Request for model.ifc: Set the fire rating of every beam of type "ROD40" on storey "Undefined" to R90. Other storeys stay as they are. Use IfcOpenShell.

First a look at what the model holds.

```python
import ifcopenshell
import ifcopenshell.util.element

model = ifcopenshell.open("model.ifc")
print(model.schema)
storey = next(s for s in model.by_type("IfcBuildingStorey") if s.Name == "Undefined")
beams = [e for e in ifcopenshell.util.element.get_decomposition(storey) if e.is_a("IfcBeam")]
seen = {}
for e in beams:
    element_type = ifcopenshell.util.element.get_type(e)
    key = (element_type.Name if element_type != e and element_type else None, ifcopenshell.util.element.get_pset(e, "Pset_BeamCommon", "FireRating"))
    seen[key] = seen.get(key, 0) + 1
for (name, value), count in sorted(seen.items(), key=str):
    print(count, "x", name, "|", value)
```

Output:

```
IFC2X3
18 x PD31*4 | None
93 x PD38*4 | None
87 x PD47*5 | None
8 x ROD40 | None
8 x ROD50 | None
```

```python
import ifcopenshell
import ifcopenshell.api.pset
import ifcopenshell.util.element

model = ifcopenshell.open("model.ifc")

storey = next(s for s in model.by_type("IfcBuildingStorey") if s.Name == "Undefined")
beams = [e for e in ifcopenshell.util.element.get_decomposition(storey) if e.is_a("IfcBeam")]

count = 0
for e in beams:
    element_type = ifcopenshell.util.element.get_type(e)
    if element_type in (None, e) or element_type.Name != "ROD40":
        continue
    found = ifcopenshell.util.element.get_pset(e, "Pset_BeamCommon", should_inherit=False)
    if found:
        pset = model.by_id(found["id"])
        if len(ifcopenshell.util.element.get_elements_by_pset(pset)) > 1:
            pset = ifcopenshell.api.pset.unshare_pset(model, products=[e], pset=pset)[0]
    else:
        pset = ifcopenshell.api.pset.add_pset(model, product=e, name="Pset_BeamCommon")
    ifcopenshell.api.pset.edit_pset(model, pset=pset, properties={"FireRating": "R90"})
    count += 1

print(count, "beams updated")

model.write("model-out.ifc")
```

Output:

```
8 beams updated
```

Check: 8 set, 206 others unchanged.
